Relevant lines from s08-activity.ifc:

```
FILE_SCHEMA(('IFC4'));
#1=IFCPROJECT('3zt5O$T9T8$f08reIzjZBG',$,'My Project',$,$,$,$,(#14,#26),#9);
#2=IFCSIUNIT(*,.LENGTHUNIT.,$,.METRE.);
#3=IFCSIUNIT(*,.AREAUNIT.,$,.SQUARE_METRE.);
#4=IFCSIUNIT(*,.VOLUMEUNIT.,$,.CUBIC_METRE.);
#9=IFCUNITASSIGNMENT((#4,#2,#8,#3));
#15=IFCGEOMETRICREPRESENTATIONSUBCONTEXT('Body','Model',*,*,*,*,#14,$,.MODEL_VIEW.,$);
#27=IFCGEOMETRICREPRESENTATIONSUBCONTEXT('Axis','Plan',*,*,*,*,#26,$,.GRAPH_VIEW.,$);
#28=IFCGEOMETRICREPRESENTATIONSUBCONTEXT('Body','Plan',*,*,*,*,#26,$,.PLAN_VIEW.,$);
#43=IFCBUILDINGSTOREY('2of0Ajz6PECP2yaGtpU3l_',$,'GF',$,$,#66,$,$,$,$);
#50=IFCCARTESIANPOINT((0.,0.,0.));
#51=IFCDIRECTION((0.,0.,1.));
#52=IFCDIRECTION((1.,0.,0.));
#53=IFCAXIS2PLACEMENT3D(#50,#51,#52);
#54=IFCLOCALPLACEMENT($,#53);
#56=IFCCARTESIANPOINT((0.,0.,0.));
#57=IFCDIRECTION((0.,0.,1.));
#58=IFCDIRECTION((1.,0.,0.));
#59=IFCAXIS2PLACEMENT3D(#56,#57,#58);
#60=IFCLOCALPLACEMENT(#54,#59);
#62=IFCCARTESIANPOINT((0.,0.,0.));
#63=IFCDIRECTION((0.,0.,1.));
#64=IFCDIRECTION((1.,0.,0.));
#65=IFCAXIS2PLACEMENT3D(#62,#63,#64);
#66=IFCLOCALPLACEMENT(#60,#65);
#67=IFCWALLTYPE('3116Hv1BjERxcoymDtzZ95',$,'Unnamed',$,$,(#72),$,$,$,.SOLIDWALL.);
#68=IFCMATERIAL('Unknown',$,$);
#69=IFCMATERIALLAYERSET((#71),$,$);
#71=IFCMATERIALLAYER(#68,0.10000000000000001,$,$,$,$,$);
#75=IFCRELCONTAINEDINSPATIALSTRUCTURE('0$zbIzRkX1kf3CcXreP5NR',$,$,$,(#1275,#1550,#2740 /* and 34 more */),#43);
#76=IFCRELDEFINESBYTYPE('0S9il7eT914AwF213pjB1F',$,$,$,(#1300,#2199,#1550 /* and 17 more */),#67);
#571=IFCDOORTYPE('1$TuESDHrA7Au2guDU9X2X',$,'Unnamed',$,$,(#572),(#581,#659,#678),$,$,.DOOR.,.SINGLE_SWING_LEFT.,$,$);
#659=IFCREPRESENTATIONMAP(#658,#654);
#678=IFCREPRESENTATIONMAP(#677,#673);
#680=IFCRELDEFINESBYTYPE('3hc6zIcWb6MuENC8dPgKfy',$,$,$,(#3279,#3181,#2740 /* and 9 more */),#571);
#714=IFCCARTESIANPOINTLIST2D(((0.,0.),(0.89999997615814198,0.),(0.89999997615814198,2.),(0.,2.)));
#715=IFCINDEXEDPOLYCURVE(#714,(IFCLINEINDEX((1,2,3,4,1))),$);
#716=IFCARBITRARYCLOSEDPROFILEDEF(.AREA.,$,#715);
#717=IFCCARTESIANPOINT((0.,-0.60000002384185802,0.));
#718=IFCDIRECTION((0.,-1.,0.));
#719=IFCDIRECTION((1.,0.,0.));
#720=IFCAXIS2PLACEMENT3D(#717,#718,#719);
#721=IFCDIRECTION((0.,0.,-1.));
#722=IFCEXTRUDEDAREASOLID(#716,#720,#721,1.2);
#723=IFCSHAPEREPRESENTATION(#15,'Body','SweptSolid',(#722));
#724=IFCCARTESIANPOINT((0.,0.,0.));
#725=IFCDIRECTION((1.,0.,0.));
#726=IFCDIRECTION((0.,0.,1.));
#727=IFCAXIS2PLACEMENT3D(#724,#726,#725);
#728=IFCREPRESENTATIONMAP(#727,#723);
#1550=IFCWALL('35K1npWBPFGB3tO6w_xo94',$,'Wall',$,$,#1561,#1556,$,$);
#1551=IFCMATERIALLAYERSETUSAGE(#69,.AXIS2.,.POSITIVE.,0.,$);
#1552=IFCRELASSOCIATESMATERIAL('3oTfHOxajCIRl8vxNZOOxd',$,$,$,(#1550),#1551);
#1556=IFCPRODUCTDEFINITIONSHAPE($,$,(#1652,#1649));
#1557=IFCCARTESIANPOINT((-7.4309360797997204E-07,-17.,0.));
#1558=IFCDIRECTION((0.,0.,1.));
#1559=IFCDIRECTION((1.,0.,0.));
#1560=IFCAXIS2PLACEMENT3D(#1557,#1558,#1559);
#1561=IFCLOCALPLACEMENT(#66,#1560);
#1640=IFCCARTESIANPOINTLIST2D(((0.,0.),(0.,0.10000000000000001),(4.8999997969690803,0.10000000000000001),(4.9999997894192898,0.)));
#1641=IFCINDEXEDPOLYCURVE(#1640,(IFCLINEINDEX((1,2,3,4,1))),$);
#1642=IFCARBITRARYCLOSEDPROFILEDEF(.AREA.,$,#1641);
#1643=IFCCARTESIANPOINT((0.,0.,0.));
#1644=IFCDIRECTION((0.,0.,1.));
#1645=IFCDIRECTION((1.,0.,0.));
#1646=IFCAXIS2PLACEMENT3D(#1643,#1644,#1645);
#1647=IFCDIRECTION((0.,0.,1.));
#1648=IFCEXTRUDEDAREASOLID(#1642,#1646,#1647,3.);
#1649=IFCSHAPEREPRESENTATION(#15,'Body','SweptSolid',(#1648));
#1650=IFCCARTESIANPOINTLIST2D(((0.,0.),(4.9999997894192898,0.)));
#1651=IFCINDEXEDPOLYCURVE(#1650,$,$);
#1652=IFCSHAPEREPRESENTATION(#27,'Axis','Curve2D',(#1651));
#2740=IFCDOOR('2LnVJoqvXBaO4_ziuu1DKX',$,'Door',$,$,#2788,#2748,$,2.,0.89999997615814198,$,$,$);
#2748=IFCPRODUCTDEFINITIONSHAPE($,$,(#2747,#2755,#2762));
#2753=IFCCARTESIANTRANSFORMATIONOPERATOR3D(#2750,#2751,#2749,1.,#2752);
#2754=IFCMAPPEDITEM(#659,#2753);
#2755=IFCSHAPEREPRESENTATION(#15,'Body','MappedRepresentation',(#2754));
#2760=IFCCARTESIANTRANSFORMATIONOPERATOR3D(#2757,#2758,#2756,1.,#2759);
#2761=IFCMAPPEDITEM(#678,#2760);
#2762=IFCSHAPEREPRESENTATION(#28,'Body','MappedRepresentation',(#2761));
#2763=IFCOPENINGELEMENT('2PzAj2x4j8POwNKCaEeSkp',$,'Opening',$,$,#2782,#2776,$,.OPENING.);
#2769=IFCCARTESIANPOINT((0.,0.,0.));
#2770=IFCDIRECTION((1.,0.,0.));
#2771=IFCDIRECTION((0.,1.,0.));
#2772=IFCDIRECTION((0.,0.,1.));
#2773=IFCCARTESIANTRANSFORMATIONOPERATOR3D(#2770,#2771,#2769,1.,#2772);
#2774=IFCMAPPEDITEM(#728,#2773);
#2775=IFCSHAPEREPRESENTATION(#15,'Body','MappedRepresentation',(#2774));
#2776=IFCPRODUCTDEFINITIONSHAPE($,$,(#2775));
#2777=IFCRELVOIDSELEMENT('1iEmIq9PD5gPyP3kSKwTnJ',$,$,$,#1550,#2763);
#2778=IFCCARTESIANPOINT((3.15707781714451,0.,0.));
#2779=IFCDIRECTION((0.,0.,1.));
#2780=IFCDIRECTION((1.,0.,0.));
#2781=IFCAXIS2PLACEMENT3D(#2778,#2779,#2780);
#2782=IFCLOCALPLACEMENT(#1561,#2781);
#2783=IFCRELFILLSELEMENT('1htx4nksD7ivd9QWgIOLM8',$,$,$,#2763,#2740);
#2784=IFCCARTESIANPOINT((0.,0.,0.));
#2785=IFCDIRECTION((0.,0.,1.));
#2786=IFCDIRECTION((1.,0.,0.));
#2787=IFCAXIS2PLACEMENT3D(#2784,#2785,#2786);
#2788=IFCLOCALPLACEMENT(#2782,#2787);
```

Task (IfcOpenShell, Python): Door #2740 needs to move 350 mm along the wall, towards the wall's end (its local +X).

```python
import ifcopenshell
import ifcopenshell.api.geometry
import ifcopenshell.util.placement
import ifcopenshell.util.unit

model = ifcopenshell.open("s08-activity.ifc")
unit_scale = ifcopenshell.util.unit.calculate_unit_scale(model)

door = model.by_guid("2LnVJoqvXBaO4_ziuu1DKX")
opening = door.FillsVoids[0].RelatingOpeningElement
wall = opening.VoidsElements[0].RelatingBuildingElement

wall_matrix = ifcopenshell.util.placement.get_local_placement(wall.ObjectPlacement)
shift = wall_matrix[:3, 0] * 0.35 / unit_scale
before = ifcopenshell.util.placement.get_local_placement(door.ObjectPlacement)[:3, 3].copy()

# The door is placed relative to its opening, so it follows when the opening moves.
matrix = ifcopenshell.util.placement.get_local_placement(opening.ObjectPlacement)
matrix[:3, 3] += shift
ifcopenshell.api.geometry.edit_object_placement(
    model, product=opening, matrix=matrix, is_si=False, should_transform_children=True
)

after = ifcopenshell.util.placement.get_local_placement(door.ObjectPlacement)[:3, 3]
print("door moved by", (after - before).round(3) + 0.0)

model.write("s08-activity_v2.ifc")
```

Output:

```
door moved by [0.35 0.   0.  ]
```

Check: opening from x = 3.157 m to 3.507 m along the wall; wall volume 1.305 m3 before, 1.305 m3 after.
